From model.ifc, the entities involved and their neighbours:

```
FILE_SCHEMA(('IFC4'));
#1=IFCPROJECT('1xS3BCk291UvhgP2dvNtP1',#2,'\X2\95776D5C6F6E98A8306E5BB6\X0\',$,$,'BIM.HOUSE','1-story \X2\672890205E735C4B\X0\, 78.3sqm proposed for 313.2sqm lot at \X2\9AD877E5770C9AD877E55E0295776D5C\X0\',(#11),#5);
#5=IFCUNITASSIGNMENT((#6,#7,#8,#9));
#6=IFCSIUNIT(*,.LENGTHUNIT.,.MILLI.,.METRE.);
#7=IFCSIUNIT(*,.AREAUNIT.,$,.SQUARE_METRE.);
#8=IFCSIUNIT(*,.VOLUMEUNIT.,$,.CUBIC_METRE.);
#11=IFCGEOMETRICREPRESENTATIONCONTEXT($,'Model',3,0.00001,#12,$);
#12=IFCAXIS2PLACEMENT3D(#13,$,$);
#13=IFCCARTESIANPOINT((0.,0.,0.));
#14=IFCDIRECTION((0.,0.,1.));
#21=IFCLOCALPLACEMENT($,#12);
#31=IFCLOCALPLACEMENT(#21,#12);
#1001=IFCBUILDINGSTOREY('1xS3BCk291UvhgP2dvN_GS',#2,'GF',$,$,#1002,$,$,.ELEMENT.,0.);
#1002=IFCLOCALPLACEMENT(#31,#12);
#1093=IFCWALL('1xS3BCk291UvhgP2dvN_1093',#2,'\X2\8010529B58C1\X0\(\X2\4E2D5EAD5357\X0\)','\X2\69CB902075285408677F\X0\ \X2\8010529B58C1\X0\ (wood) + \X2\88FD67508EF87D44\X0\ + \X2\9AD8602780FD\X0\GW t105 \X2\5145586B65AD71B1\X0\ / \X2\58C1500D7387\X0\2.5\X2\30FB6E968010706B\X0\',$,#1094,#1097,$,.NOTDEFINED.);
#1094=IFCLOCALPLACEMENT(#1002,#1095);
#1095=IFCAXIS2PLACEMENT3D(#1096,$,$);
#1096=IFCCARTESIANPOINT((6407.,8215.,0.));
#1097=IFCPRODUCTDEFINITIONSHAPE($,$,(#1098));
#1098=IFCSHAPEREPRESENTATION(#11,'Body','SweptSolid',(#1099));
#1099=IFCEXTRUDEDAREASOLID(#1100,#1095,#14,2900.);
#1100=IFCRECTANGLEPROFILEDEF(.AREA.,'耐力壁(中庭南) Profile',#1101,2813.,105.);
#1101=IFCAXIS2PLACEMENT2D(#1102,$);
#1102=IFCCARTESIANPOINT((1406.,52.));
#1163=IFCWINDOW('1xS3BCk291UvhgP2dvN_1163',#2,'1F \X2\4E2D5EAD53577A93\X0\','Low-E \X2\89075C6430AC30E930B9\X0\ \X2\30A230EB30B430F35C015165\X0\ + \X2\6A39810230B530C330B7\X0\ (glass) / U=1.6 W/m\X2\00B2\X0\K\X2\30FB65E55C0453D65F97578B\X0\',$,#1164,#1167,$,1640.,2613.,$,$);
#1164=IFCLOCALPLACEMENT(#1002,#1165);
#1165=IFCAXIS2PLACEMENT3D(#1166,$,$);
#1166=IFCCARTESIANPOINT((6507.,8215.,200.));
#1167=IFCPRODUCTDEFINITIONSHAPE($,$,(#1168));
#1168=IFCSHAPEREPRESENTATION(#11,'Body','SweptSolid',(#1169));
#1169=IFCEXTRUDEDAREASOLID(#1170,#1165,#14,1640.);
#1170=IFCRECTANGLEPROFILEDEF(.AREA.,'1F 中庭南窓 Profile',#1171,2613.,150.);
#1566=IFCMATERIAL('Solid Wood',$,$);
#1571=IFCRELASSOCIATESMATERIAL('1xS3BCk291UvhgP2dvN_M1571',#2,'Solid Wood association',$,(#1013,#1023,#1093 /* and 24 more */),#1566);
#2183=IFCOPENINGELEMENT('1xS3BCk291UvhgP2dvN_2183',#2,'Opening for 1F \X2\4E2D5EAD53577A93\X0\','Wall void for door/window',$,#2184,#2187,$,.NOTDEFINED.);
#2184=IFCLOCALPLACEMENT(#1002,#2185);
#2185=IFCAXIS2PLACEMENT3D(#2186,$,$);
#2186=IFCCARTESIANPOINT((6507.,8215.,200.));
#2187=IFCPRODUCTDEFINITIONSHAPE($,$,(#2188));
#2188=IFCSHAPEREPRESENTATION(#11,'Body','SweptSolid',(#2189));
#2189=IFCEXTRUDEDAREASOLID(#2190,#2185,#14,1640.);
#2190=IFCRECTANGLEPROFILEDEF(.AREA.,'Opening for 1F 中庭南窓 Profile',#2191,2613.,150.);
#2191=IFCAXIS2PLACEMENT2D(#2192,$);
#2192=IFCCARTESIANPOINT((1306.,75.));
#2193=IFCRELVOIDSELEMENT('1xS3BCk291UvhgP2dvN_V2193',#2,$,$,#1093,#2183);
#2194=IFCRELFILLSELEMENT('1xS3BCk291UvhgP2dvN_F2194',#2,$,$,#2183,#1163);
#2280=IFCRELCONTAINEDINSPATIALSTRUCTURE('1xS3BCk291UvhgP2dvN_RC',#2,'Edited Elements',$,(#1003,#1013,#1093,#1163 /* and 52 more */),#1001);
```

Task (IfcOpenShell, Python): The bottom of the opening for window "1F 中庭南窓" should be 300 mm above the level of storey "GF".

```python
import numpy as np
import ifcopenshell
import ifcopenshell.api.geometry
import ifcopenshell.geom
import ifcopenshell.util.element
import ifcopenshell.util.placement
import ifcopenshell.util.shape
import ifcopenshell.util.unit

model = ifcopenshell.open("model.ifc")
unit_scale = ifcopenshell.util.unit.calculate_unit_scale(model)

window = model.by_id(1163)
opening = window.FillsVoids[0].RelatingOpeningElement
storey = ifcopenshell.util.element.get_container(window, ifc_class="IfcBuildingStorey")
level = ifcopenshell.util.placement.get_local_placement(storey.ObjectPlacement)[2, 3]

# The opening's origin need not be at the sill, so measure its lowest point.
shape = ifcopenshell.geom.create_shape(ifcopenshell.geom.settings(), opening)
bottom = ifcopenshell.util.shape.get_shape_bottom_elevation(shape, shape.geometry) / unit_scale
dz = level + 0.3 / unit_scale - bottom

shift = np.array([0.0, 0.0, dz])
# The window is not placed relative to its opening, so move both.
for product in (opening, window):
    matrix = ifcopenshell.util.placement.get_local_placement(product.ObjectPlacement)
    matrix[:3, 3] += shift
    ifcopenshell.api.geometry.edit_object_placement(model, product=product, matrix=matrix, is_si=False)

print(f"moved by {dz * unit_scale:+.3f} m")

model.write("model_v2.ifc")
```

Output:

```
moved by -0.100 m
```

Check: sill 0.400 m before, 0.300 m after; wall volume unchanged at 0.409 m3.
